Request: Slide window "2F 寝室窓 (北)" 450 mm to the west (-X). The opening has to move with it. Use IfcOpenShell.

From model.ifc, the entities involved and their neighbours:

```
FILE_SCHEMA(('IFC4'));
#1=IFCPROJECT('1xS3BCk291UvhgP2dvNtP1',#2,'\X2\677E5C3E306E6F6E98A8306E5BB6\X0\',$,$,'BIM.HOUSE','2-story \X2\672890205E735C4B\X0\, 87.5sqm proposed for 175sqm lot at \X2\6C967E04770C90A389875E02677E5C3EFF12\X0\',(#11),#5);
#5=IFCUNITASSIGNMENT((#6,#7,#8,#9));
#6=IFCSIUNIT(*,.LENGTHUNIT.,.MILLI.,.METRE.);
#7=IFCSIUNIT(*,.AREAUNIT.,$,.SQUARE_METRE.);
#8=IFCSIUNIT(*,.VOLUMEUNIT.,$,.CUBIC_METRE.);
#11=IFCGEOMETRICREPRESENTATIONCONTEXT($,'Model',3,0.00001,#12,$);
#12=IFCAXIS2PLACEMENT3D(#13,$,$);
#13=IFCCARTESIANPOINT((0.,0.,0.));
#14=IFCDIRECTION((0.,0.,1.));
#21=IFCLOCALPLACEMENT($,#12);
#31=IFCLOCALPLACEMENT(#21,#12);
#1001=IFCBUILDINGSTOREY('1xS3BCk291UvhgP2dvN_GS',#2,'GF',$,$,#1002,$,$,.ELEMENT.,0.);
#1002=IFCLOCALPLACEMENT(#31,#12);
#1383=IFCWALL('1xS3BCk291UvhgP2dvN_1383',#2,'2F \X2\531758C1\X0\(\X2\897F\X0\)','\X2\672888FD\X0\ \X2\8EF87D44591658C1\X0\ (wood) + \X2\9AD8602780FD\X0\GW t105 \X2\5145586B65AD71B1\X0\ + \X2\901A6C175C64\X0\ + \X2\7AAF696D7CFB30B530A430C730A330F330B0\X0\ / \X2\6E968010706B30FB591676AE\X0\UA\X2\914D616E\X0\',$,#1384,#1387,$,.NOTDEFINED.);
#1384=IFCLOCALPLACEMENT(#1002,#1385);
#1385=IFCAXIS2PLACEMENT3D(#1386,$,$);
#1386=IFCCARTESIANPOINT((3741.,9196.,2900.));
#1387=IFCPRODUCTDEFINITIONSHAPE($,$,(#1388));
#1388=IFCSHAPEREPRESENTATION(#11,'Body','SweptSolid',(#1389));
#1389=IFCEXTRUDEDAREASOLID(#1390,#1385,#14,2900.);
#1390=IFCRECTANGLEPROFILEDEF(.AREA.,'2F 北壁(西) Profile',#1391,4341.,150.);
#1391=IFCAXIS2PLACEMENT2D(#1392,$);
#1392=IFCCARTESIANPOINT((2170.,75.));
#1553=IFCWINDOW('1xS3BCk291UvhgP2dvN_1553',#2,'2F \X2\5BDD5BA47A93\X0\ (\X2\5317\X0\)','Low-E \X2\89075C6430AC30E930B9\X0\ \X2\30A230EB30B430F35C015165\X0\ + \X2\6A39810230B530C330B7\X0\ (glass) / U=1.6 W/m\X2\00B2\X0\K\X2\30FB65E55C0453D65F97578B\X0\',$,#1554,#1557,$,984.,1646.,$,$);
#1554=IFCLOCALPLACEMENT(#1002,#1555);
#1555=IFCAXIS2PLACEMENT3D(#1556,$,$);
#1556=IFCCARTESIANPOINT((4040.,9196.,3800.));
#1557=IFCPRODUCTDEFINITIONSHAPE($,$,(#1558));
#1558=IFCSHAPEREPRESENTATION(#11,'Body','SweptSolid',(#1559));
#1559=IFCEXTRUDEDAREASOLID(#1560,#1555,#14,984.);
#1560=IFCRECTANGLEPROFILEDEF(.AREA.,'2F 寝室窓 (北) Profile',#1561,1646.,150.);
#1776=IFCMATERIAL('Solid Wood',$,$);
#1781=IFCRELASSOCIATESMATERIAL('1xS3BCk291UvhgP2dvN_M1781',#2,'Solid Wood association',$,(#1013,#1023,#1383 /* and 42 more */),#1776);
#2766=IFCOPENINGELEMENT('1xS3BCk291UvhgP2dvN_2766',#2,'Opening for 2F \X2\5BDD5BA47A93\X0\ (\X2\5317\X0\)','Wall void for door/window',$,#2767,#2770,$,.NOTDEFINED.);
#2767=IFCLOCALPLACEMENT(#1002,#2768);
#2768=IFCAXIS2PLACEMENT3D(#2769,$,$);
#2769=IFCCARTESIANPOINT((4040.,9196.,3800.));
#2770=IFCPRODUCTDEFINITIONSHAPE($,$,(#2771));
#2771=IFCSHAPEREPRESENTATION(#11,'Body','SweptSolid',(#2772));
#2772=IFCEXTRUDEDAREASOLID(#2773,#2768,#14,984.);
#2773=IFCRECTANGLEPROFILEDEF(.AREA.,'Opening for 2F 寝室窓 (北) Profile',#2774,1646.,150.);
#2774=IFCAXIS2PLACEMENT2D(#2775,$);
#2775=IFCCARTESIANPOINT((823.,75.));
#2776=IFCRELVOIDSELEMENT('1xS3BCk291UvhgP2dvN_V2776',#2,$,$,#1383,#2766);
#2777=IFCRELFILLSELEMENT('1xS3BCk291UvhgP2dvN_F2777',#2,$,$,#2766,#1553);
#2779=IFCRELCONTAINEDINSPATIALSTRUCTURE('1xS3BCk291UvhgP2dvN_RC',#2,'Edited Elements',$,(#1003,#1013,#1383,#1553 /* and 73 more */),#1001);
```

```python
import ifcopenshell
import ifcopenshell.api.geometry
import ifcopenshell.util.placement
import ifcopenshell.util.unit

model = ifcopenshell.open("model.ifc")
unit_scale = ifcopenshell.util.unit.calculate_unit_scale(model)

window = model.by_guid("1xS3BCk291UvhgP2dvN_1553")
opening = window.FillsVoids[0].RelatingOpeningElement
wall = opening.VoidsElements[0].RelatingBuildingElement

wall_matrix = ifcopenshell.util.placement.get_local_placement(wall.ObjectPlacement)
shift = wall_matrix[:3, 0] * -0.45 / unit_scale
before = ifcopenshell.util.placement.get_local_placement(window.ObjectPlacement)[:3, 3].copy()

# The window is not placed relative to its opening, so move both.
for product in (opening, window):
    matrix = ifcopenshell.util.placement.get_local_placement(product.ObjectPlacement)
    matrix[:3, 3] += shift
    ifcopenshell.api.geometry.edit_object_placement(model, product=product, matrix=matrix, is_si=False)

after = ifcopenshell.util.placement.get_local_placement(window.ObjectPlacement)[:3, 3]
print("window moved by", (after - before).round(3) + 0.0)

model.write("model_v2.ifc")
```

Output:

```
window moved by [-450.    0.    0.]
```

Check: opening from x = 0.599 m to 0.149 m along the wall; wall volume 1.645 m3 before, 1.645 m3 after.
